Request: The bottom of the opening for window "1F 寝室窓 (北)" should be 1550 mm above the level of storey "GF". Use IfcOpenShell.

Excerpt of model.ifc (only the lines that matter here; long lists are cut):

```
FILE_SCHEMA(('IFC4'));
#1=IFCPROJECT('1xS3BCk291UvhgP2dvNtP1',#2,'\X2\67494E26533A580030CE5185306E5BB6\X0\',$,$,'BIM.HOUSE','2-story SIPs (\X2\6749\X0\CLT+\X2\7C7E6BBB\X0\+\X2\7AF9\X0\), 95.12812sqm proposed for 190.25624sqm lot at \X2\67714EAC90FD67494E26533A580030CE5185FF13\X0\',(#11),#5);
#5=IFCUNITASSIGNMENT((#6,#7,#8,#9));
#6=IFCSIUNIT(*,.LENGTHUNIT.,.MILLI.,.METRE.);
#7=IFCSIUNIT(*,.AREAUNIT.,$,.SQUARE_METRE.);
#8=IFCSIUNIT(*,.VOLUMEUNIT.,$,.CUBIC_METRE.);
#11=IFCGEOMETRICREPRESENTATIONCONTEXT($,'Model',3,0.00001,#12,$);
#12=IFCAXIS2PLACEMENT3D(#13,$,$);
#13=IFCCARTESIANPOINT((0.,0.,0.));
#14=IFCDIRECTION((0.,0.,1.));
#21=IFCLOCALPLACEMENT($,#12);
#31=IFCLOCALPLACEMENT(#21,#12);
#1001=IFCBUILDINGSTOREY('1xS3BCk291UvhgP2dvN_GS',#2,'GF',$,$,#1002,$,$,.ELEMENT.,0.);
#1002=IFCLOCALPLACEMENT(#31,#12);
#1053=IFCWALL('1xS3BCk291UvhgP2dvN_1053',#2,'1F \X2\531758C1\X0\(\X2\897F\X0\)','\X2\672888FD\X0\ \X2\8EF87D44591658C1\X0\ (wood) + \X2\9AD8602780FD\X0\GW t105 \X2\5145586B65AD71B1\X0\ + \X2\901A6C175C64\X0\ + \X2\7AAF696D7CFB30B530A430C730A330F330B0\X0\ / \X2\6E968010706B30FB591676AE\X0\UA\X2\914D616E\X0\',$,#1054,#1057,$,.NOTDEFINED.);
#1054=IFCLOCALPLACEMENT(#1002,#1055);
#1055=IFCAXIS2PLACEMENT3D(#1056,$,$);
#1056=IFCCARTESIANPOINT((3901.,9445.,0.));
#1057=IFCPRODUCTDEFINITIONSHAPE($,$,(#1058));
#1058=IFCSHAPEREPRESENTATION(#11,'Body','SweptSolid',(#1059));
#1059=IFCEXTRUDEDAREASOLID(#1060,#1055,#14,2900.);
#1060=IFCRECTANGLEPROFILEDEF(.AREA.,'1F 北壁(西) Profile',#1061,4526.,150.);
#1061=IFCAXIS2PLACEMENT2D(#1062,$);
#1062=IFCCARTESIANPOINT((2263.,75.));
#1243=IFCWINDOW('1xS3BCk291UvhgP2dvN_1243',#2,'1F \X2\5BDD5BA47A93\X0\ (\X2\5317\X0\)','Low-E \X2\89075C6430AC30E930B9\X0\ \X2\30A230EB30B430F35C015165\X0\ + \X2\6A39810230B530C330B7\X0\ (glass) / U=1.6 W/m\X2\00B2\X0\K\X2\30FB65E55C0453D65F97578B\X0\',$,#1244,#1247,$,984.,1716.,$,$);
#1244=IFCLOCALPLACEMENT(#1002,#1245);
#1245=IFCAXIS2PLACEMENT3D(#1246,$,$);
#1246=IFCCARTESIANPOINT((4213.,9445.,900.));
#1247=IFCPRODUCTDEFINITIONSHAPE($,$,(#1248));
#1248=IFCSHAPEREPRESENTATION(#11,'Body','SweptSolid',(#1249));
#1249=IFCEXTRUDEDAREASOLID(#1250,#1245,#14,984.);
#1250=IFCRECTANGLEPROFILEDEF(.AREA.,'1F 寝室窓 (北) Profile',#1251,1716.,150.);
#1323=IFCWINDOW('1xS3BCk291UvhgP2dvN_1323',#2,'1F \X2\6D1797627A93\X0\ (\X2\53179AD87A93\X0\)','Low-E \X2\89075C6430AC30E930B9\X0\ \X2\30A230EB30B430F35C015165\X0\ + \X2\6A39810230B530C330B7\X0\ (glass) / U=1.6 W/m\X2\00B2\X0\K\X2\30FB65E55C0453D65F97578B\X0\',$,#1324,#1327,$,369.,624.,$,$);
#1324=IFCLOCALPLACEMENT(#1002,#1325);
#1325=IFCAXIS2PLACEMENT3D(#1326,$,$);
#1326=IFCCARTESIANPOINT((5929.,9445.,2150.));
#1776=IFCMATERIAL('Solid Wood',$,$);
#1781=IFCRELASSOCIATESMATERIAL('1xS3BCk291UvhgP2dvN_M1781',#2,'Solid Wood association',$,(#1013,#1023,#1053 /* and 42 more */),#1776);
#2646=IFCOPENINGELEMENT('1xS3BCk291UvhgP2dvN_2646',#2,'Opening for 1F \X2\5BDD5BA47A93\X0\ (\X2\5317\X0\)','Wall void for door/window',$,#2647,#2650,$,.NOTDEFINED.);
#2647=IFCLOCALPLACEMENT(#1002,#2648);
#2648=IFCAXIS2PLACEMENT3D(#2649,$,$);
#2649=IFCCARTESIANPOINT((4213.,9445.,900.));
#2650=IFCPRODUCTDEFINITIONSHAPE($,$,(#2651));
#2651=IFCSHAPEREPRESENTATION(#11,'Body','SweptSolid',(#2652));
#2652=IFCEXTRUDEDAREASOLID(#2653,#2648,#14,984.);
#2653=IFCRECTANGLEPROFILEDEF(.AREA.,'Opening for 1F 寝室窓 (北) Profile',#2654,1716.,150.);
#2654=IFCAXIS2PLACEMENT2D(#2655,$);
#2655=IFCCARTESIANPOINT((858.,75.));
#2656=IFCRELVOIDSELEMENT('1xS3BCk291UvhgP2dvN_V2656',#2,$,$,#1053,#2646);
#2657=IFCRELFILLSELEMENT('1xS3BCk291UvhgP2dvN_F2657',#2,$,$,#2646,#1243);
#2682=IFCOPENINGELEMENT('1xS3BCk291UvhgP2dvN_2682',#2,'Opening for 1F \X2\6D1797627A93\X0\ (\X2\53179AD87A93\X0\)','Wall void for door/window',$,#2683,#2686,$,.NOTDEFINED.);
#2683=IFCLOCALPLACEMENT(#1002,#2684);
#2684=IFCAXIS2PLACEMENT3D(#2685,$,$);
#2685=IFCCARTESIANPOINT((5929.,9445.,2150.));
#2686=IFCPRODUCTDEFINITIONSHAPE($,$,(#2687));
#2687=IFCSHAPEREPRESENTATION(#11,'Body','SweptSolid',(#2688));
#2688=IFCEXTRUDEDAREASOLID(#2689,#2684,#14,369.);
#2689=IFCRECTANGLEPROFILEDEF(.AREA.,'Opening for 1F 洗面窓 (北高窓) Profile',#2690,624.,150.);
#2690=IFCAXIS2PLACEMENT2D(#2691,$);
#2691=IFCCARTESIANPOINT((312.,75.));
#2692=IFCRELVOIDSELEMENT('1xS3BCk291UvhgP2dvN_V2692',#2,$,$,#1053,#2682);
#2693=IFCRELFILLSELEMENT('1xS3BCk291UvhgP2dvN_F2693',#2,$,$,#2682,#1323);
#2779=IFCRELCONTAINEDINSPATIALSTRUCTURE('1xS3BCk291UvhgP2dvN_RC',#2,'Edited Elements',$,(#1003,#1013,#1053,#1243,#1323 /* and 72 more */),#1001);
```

```python
import numpy as np
import ifcopenshell
import ifcopenshell.api.geometry
import ifcopenshell.geom
import ifcopenshell.util.element
import ifcopenshell.util.placement
import ifcopenshell.util.shape
import ifcopenshell.util.unit

model = ifcopenshell.open("model.ifc")
unit_scale = ifcopenshell.util.unit.calculate_unit_scale(model)

window = model.by_guid("1xS3BCk291UvhgP2dvN_1243")
opening = window.FillsVoids[0].RelatingOpeningElement
storey = ifcopenshell.util.element.get_container(window, ifc_class="IfcBuildingStorey")
level = ifcopenshell.util.placement.get_local_placement(storey.ObjectPlacement)[2, 3]

# The opening's origin need not be at the sill, so measure its lowest point.
shape = ifcopenshell.geom.create_shape(ifcopenshell.geom.settings(), opening)
bottom = ifcopenshell.util.shape.get_shape_bottom_elevation(shape, shape.geometry) / unit_scale
dz = level + 1550.0 - bottom

shift = np.array([0.0, 0.0, dz])
# The window is not placed relative to its opening, so move both.
for product in (opening, window):
    matrix = ifcopenshell.util.placement.get_local_placement(product.ObjectPlacement)
    matrix[:3, 3] += shift
    ifcopenshell.api.geometry.edit_object_placement(model, product=product, matrix=matrix, is_si=False)

print(f"moved by {dz * unit_scale:+.3f} m")

model.write("model-out.ifc")
```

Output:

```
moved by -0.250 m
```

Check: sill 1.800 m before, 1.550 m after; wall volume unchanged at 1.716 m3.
